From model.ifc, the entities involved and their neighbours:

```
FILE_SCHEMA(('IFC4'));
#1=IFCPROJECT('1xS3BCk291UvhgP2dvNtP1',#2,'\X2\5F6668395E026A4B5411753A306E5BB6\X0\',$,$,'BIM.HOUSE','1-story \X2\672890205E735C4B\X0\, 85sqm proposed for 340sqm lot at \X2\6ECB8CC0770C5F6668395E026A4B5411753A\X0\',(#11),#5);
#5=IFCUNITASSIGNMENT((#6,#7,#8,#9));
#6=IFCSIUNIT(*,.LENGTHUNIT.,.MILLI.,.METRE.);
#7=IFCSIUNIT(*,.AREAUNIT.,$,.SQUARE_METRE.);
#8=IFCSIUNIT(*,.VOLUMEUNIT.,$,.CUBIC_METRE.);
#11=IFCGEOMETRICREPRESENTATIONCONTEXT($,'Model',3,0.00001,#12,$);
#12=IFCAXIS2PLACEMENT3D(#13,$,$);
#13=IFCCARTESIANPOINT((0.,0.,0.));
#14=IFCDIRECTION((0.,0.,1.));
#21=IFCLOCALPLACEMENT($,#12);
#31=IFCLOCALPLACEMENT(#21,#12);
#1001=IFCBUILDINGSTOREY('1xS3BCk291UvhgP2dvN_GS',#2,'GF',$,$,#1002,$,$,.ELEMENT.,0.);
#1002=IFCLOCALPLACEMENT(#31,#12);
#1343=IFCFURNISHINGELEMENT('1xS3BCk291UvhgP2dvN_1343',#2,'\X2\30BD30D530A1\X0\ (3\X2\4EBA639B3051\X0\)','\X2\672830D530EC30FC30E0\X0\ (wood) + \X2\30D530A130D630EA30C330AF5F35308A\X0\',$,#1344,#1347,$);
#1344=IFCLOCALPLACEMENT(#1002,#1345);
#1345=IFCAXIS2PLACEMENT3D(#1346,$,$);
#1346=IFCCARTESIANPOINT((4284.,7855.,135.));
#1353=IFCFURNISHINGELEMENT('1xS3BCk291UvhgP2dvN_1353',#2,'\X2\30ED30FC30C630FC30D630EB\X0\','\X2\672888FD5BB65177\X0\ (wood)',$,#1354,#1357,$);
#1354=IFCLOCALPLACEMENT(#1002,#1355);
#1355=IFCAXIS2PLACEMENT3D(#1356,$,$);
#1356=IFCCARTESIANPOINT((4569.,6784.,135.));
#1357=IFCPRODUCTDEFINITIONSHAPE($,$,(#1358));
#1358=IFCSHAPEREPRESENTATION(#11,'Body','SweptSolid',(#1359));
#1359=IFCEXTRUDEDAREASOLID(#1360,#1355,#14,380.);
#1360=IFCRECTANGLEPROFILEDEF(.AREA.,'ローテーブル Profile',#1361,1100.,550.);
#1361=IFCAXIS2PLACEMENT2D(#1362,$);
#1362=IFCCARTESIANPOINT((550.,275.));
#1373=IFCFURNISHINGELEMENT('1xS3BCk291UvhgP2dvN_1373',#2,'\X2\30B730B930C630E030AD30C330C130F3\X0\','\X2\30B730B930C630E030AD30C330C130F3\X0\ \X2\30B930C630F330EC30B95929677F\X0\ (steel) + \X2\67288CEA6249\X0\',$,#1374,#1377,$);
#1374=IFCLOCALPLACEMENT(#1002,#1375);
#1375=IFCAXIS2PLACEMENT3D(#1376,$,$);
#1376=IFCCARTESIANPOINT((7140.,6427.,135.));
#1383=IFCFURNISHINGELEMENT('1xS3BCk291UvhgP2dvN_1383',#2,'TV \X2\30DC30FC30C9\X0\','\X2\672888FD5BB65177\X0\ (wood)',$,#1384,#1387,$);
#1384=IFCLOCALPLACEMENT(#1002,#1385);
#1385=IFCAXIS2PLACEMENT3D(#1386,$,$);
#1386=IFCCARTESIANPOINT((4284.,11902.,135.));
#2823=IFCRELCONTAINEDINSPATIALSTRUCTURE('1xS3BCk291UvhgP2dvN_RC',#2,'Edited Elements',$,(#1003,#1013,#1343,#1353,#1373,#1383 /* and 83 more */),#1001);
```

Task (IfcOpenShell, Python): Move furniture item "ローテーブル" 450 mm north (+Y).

```python
import ifcopenshell
import ifcopenshell.api.geometry
import ifcopenshell.util.placement
import ifcopenshell.util.unit

model = ifcopenshell.open("model.ifc")
unit_scale = ifcopenshell.util.unit.calculate_unit_scale(model)

item = model.by_guid("1xS3BCk291UvhgP2dvN_1353")
matrix = ifcopenshell.util.placement.get_local_placement(item.ObjectPlacement)
matrix[1, 3] += 0.45 / unit_scale
ifcopenshell.api.geometry.edit_object_placement(model, product=item, matrix=matrix, is_si=False)

print(ifcopenshell.util.placement.get_local_placement(item.ObjectPlacement).round(3) + 0.0)

model.write("model_updated.ifc")
```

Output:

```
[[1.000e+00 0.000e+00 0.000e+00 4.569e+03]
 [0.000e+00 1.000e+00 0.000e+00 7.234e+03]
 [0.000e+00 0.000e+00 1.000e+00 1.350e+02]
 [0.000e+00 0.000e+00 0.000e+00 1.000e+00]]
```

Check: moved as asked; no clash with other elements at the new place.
